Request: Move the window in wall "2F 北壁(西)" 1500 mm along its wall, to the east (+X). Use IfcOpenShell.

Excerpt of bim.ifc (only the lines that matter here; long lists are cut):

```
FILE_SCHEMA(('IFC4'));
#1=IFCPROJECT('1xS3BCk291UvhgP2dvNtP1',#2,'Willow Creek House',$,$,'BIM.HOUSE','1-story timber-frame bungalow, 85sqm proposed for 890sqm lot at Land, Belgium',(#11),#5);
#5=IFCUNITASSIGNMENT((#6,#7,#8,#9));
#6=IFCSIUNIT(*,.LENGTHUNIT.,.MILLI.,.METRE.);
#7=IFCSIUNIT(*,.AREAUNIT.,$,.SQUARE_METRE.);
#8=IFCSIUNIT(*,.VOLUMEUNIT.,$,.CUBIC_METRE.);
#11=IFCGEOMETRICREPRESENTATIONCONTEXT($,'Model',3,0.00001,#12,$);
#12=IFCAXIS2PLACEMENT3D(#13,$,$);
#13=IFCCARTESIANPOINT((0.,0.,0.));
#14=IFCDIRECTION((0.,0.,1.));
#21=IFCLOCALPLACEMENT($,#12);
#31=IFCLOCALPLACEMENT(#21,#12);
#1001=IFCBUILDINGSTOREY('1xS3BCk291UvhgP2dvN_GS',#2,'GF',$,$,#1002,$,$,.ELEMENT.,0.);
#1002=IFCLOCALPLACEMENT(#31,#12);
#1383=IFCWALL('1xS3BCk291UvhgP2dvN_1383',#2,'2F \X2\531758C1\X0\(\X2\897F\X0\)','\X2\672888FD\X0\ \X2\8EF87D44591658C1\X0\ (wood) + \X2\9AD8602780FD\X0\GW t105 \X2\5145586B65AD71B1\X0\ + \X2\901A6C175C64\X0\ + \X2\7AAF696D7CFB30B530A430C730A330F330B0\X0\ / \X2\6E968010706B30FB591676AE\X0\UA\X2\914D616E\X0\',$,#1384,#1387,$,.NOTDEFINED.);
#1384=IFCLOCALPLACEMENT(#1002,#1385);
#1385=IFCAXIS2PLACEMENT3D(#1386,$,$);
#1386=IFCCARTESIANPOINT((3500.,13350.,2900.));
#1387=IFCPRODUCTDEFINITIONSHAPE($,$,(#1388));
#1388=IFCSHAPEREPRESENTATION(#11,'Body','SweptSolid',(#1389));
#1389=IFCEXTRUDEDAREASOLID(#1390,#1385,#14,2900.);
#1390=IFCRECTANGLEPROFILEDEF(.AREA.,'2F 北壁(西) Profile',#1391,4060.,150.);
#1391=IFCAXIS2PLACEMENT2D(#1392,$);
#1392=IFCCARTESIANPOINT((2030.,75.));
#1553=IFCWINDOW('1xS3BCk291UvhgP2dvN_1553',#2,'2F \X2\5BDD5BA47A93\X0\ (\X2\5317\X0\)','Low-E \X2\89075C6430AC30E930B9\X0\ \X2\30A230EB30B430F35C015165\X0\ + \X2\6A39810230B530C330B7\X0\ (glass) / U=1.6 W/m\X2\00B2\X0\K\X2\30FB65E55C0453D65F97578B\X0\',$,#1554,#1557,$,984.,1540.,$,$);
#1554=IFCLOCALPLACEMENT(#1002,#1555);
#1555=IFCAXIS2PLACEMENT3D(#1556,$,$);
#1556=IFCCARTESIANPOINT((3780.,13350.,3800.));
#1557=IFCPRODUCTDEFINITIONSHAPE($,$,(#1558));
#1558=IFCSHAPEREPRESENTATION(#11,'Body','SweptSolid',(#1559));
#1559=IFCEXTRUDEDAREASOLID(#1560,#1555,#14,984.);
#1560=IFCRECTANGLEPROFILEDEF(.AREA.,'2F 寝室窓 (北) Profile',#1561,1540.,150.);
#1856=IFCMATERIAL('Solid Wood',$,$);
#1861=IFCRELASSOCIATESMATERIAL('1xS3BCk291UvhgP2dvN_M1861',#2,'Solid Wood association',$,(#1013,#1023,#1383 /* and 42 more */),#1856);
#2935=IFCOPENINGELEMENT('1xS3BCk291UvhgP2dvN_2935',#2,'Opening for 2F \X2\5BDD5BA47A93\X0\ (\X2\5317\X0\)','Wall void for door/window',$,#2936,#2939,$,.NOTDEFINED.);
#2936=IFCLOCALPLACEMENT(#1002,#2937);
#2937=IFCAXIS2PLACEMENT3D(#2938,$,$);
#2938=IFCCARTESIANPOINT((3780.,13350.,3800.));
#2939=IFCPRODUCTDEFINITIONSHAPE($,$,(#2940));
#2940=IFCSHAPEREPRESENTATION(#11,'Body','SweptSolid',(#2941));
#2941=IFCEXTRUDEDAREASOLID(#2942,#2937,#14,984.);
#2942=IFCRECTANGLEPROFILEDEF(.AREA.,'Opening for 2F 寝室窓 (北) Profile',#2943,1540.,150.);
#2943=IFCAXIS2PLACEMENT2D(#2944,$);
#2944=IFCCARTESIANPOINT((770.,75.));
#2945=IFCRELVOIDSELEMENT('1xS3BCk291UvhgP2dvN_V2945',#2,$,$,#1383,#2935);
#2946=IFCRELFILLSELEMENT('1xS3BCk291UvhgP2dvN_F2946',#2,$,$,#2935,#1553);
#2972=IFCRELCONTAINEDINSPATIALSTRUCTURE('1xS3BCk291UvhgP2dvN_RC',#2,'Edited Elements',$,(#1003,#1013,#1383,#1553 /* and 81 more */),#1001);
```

```python
import ifcopenshell
import ifcopenshell.api.geometry
import ifcopenshell.util.placement

model = ifcopenshell.open("bim.ifc")

window = model.by_id(1553)
opening = window.FillsVoids[0].RelatingOpeningElement
wall = opening.VoidsElements[0].RelatingBuildingElement

wall_matrix = ifcopenshell.util.placement.get_local_placement(wall.ObjectPlacement)
shift = wall_matrix[:3, 0] * 1500.0
before = ifcopenshell.util.placement.get_local_placement(window.ObjectPlacement)[:3, 3].copy()

# The window is not placed relative to its opening, so move both.
for product in (opening, window):
    matrix = ifcopenshell.util.placement.get_local_placement(product.ObjectPlacement)
    matrix[:3, 3] += shift
    ifcopenshell.api.geometry.edit_object_placement(model, product=product, matrix=matrix, is_si=False)

after = ifcopenshell.util.placement.get_local_placement(window.ObjectPlacement)[:3, 3]
print("window moved by", (after - before).round(3) + 0.0)

model.write("bim_v2.ifc")
```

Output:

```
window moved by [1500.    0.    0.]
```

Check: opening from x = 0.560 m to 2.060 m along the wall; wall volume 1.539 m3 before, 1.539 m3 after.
